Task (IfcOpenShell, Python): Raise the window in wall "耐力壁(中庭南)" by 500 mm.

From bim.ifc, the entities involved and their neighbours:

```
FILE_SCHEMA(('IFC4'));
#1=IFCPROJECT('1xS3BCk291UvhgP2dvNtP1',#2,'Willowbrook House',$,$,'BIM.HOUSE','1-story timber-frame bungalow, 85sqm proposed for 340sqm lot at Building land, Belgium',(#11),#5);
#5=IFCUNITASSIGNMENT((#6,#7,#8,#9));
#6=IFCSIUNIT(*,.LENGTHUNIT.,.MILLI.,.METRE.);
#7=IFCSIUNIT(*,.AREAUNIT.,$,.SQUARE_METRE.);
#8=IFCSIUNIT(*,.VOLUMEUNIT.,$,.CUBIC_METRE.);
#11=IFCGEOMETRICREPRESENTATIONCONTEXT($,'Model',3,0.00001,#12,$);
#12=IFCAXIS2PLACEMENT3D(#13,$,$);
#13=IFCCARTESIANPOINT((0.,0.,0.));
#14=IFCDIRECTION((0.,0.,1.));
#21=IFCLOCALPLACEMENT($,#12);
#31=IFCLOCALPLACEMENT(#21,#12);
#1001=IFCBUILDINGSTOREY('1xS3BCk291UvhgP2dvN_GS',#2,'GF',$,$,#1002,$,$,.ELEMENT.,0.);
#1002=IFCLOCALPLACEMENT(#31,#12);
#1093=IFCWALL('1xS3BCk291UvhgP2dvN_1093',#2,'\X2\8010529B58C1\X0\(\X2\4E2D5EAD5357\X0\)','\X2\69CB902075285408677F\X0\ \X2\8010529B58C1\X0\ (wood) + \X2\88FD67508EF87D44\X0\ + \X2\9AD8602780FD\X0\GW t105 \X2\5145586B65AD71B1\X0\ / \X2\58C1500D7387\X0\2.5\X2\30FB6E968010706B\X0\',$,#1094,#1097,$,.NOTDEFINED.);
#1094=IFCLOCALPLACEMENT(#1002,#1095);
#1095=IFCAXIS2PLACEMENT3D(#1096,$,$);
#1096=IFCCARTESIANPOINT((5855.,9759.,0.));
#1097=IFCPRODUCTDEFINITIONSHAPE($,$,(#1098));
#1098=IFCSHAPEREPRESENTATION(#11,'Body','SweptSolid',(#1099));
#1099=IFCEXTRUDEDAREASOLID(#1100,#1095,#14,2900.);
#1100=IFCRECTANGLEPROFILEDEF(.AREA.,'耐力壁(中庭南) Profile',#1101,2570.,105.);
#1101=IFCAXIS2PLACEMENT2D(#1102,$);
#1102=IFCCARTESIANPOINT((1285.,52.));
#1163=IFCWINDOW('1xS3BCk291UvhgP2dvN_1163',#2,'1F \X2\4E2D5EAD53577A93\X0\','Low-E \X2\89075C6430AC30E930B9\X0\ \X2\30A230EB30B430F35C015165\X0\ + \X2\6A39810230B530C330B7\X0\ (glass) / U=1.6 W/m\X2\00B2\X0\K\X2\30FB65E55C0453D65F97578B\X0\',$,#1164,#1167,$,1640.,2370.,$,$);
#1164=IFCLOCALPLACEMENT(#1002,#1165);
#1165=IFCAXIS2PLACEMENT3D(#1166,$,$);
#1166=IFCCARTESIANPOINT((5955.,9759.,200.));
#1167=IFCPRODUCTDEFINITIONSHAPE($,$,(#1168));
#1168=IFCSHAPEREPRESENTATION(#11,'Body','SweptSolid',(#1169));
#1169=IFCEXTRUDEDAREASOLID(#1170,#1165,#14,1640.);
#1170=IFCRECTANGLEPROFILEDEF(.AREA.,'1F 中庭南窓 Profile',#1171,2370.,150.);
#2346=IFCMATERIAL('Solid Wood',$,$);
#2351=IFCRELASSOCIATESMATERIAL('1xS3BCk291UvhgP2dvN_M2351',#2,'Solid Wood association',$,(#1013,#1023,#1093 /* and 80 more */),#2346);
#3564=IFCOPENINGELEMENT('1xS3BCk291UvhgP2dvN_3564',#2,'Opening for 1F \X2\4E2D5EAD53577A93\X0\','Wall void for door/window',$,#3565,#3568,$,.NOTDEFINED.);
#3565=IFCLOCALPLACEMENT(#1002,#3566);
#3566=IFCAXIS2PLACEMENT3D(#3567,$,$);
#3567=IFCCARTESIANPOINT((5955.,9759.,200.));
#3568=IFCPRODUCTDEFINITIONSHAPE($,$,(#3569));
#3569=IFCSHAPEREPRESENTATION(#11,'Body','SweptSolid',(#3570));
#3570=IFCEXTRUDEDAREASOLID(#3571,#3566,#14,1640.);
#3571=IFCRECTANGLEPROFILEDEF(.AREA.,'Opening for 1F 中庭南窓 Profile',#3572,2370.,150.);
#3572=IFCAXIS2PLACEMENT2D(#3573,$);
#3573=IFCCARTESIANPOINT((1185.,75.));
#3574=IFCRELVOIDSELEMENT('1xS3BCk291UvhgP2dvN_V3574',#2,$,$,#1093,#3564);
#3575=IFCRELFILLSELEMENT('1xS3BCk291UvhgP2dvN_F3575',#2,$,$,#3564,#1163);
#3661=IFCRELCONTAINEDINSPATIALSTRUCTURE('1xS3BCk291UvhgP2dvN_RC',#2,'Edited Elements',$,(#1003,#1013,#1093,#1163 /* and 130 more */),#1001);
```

```python
import numpy as np
import ifcopenshell
import ifcopenshell.api.geometry
import ifcopenshell.util.placement
import ifcopenshell.util.unit

model = ifcopenshell.open("bim.ifc")
unit_scale = ifcopenshell.util.unit.calculate_unit_scale(model)

window = model.by_guid("1xS3BCk291UvhgP2dvN_1163")
opening = window.FillsVoids[0].RelatingOpeningElement
dz = 0.5 / unit_scale

shift = np.array([0.0, 0.0, dz])
# The window is not placed relative to its opening, so move both.
for product in (opening, window):
    matrix = ifcopenshell.util.placement.get_local_placement(product.ObjectPlacement)
    matrix[:3, 3] += shift
    ifcopenshell.api.geometry.edit_object_placement(model, product=product, matrix=matrix, is_si=False)

print(f"moved by {dz * unit_scale:+.3f} m")

model.write("bim_edited.ifc")
```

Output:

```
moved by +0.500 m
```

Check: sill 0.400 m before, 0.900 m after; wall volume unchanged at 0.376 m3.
